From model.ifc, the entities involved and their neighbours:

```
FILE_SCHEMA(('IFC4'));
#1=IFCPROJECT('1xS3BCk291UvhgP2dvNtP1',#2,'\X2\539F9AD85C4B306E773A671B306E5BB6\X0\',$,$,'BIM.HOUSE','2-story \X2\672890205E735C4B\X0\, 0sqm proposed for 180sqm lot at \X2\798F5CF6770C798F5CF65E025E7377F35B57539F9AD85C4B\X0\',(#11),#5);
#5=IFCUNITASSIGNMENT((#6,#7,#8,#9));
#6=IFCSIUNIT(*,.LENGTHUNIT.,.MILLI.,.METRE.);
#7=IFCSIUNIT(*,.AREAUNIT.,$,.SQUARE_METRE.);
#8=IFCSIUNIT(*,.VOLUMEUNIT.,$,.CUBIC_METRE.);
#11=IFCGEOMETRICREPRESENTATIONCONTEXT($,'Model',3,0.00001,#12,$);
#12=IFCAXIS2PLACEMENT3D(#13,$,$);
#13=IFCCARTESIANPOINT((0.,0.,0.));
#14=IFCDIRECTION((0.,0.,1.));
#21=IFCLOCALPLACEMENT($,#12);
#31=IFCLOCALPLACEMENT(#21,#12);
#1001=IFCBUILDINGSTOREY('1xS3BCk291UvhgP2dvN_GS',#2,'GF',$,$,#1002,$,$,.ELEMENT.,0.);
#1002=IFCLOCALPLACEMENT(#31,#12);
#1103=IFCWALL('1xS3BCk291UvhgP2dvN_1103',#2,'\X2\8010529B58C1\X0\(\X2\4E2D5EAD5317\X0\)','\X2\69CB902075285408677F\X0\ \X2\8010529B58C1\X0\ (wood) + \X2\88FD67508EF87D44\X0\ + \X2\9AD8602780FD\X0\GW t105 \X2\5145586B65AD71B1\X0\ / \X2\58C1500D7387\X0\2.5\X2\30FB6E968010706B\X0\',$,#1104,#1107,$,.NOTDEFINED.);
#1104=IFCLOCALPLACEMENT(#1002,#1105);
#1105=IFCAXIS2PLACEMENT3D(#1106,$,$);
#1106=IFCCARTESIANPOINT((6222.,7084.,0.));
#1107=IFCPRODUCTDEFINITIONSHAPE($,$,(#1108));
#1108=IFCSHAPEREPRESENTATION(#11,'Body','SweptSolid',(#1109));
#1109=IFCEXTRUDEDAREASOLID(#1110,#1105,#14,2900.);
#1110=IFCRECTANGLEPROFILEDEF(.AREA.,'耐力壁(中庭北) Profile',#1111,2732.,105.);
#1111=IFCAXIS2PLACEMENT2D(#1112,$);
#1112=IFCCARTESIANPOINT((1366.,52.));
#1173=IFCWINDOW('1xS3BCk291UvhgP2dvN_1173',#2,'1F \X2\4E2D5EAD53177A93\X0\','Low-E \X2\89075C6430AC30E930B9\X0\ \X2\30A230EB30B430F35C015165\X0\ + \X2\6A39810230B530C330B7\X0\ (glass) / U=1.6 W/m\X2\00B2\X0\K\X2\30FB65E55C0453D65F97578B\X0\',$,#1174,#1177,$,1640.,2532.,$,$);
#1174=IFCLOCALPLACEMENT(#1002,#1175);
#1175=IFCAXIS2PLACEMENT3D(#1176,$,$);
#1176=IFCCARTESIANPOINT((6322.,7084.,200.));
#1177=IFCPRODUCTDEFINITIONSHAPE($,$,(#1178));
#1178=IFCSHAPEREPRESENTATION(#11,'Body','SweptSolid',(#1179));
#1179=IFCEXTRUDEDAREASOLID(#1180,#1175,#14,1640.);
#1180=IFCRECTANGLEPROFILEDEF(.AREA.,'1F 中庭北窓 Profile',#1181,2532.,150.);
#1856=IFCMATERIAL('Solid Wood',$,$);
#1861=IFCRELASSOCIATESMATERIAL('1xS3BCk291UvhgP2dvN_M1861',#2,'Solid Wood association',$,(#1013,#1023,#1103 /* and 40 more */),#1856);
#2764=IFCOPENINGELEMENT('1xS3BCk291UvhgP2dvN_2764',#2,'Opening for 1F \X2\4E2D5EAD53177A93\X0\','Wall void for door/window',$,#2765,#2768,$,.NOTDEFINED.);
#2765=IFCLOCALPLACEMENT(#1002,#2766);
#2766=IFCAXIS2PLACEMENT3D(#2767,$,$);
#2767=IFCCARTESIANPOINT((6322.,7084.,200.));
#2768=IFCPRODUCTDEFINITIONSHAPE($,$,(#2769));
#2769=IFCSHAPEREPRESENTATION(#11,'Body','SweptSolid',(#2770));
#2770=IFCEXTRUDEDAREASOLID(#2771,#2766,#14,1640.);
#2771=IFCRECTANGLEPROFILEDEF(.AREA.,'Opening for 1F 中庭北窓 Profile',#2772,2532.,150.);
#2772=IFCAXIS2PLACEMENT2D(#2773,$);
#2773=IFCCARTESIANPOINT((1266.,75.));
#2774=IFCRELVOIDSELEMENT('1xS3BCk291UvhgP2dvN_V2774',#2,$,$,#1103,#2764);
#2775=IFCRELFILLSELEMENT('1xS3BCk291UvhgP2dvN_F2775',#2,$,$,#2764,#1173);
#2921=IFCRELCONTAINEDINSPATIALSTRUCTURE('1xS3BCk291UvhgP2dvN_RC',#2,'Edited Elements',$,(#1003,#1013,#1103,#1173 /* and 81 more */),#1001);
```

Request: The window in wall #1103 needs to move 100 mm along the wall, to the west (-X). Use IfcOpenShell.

```python
import ifcopenshell
import ifcopenshell.api.geometry
import ifcopenshell.util.placement
import ifcopenshell.util.unit

model = ifcopenshell.open("model.ifc")
unit_scale = ifcopenshell.util.unit.calculate_unit_scale(model)

window = model.by_guid("1xS3BCk291UvhgP2dvN_1173")
opening = window.FillsVoids[0].RelatingOpeningElement
wall = opening.VoidsElements[0].RelatingBuildingElement

wall_matrix = ifcopenshell.util.placement.get_local_placement(wall.ObjectPlacement)
shift = wall_matrix[:3, 0] * -0.1 / unit_scale
before = ifcopenshell.util.placement.get_local_placement(window.ObjectPlacement)[:3, 3].copy()

# The window is not placed relative to its opening, so move both.
for product in (opening, window):
    matrix = ifcopenshell.util.placement.get_local_placement(product.ObjectPlacement)
    matrix[:3, 3] += shift
    ifcopenshell.api.geometry.edit_object_placement(model, product=product, matrix=matrix, is_si=False)

after = ifcopenshell.util.placement.get_local_placement(window.ObjectPlacement)[:3, 3]
print("window moved by", (after - before).round(3) + 0.0)

model.write("model-out.ifc")
```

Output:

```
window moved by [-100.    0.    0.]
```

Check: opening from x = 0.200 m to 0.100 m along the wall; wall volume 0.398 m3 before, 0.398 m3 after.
